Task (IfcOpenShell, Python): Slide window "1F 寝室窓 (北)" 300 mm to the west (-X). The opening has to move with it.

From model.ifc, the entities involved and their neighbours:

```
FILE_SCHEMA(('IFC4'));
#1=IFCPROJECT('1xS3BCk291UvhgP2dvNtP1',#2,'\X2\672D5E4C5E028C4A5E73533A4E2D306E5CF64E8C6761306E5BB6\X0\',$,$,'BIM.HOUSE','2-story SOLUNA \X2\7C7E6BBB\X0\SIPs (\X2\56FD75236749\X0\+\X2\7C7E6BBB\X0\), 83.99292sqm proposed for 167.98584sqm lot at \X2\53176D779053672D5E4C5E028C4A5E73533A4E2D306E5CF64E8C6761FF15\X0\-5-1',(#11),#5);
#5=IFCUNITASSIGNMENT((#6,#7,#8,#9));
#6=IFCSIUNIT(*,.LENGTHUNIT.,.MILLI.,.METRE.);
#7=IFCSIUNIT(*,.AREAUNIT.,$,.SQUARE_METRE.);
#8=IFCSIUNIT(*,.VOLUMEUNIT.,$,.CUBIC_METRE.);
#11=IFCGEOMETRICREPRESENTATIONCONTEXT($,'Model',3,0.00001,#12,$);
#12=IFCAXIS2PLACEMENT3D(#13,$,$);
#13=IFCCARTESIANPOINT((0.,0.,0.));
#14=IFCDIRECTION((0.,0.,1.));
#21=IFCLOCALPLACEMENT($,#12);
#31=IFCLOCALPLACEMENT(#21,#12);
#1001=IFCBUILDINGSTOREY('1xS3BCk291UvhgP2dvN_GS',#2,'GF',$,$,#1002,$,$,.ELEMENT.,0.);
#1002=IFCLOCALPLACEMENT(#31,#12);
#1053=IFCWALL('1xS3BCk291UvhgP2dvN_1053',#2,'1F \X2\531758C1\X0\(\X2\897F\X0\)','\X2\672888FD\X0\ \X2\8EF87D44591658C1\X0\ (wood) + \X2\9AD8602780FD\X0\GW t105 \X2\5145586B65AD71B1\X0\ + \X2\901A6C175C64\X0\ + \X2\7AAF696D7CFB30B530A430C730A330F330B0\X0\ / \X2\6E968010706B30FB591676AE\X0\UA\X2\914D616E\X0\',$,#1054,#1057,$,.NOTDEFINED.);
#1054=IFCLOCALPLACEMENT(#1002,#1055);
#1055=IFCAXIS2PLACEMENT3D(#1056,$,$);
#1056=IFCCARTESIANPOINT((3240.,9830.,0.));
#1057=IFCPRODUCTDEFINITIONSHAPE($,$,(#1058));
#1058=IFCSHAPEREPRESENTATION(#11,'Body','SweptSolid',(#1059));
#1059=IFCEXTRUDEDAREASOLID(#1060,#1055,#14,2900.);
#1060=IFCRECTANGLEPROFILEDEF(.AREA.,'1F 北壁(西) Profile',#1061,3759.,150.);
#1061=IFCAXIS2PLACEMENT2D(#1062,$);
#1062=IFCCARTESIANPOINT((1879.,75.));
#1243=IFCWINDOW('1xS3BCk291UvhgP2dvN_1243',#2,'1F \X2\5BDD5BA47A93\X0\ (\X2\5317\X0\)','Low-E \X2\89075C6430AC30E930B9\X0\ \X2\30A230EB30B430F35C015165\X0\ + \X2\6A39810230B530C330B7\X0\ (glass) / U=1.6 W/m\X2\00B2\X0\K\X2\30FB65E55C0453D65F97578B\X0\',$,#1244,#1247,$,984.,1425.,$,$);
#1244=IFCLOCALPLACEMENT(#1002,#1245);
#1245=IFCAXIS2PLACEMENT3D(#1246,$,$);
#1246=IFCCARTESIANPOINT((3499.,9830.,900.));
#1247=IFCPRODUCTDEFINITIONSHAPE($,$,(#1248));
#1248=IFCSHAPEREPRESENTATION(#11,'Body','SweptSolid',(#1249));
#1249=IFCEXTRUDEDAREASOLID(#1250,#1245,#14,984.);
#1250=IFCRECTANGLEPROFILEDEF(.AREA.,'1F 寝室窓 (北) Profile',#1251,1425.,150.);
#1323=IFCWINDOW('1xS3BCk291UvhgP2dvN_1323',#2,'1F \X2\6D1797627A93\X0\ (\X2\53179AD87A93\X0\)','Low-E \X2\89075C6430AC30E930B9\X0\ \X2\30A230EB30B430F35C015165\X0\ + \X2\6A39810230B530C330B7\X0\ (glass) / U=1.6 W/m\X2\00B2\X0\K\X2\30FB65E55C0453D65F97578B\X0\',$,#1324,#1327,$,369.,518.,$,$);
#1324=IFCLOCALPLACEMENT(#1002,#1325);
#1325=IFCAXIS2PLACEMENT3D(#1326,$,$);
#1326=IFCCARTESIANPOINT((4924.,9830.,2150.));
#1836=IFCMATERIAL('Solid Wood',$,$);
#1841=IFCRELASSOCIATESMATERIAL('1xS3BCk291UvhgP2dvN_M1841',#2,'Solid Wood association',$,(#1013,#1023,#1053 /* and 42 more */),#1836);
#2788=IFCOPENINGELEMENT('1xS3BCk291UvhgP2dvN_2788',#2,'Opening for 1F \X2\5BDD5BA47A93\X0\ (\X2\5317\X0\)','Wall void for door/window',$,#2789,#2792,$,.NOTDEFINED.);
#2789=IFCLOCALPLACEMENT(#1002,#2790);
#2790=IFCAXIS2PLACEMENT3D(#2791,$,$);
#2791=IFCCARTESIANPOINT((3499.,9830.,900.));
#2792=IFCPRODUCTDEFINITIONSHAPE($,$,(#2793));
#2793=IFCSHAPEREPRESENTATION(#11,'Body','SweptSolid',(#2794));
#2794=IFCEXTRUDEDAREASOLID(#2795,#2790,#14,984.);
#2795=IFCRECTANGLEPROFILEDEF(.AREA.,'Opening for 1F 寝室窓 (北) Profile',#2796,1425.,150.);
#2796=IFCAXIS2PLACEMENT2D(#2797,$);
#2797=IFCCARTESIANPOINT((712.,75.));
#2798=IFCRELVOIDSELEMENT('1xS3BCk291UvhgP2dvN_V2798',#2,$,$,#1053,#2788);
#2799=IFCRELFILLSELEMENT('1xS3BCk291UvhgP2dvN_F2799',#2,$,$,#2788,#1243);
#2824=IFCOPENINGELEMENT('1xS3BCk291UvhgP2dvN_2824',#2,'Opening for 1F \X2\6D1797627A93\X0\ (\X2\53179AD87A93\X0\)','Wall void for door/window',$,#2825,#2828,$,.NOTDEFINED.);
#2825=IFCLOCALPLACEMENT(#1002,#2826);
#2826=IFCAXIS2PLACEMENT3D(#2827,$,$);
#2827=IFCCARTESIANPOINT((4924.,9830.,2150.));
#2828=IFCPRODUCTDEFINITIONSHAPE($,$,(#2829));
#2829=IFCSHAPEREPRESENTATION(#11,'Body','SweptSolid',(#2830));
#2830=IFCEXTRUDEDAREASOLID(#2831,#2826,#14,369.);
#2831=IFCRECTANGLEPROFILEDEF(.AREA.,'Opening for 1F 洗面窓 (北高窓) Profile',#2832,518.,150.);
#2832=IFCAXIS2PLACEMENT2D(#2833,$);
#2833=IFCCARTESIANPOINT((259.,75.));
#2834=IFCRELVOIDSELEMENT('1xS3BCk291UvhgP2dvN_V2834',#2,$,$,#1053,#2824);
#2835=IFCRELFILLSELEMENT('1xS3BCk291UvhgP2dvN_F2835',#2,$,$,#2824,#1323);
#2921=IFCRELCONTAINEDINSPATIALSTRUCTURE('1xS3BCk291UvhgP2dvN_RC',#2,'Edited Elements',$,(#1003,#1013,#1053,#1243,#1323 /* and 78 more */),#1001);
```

```python
import ifcopenshell
import ifcopenshell.api.geometry
import ifcopenshell.util.placement
import ifcopenshell.util.unit

model = ifcopenshell.open("model.ifc")
unit_scale = ifcopenshell.util.unit.calculate_unit_scale(model)

window = model.by_guid("1xS3BCk291UvhgP2dvN_1243")
opening = window.FillsVoids[0].RelatingOpeningElement
wall = opening.VoidsElements[0].RelatingBuildingElement

wall_matrix = ifcopenshell.util.placement.get_local_placement(wall.ObjectPlacement)
shift = wall_matrix[:3, 0] * -0.3 / unit_scale
before = ifcopenshell.util.placement.get_local_placement(window.ObjectPlacement)[:3, 3].copy()

# The window is not placed relative to its opening, so move both.
for product in (opening, window):
    matrix = ifcopenshell.util.placement.get_local_placement(product.ObjectPlacement)
    matrix[:3, 3] += shift
    ifcopenshell.api.geometry.edit_object_placement(model, product=product, matrix=matrix, is_si=False)

after = ifcopenshell.util.placement.get_local_placement(window.ObjectPlacement)[:3, 3]
print("window moved by", (after - before).round(3) + 0.0)

model.write("model_v2.ifc")
```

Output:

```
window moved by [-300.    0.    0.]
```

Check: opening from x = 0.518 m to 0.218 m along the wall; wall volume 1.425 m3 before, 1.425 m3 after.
